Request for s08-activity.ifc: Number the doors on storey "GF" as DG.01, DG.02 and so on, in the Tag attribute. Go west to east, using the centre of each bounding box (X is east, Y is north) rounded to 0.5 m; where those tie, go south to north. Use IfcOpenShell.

First a look at what the model holds.

```python
import ifcopenshell
import ifcopenshell.util.element
import ifcopenshell.util.placement

model = ifcopenshell.open("s08-activity.ifc")
print(model.schema)
storey = next(s for s in model.by_type("IfcBuildingStorey") if s.Name == "GF")
doors = [e for e in ifcopenshell.util.element.get_decomposition(storey) if e.is_a("IfcDoor")]
for e in sorted(doors, key=lambda e: e.id()):
    origin = ifcopenshell.util.placement.get_local_placement(e.ObjectPlacement)[:3, 3]
    print(e.id(), e.Tag, e.Name, origin.round(2) + 0.0, sep=" | ")
```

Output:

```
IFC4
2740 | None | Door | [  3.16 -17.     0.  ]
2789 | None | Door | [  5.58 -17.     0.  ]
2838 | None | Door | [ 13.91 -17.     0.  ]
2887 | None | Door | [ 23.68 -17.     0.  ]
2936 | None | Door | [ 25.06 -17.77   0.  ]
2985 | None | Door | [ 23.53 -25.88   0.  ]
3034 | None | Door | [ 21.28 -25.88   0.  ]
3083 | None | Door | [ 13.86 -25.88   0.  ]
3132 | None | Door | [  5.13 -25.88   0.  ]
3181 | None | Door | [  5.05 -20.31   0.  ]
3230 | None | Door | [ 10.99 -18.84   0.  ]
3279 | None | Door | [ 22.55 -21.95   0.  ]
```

```python
import ifcopenshell
import ifcopenshell.geom
import ifcopenshell.util.element
import ifcopenshell.util.shape

model = ifcopenshell.open("s08-activity.ifc")
settings = ifcopenshell.geom.settings()
settings.set("use-world-coords", True)


def centre(element):
    shape = ifcopenshell.geom.create_shape(settings, element)
    return ifcopenshell.util.shape.get_bbox_centroid(shape.geometry)


storey = next(s for s in model.by_type("IfcBuildingStorey") if s.Name == "GF")
doors = [e for e in ifcopenshell.util.element.get_decomposition(storey) if e.is_a("IfcDoor")]

# Insertion points can sit at a corner or the storey origin, so sort by the geometry (in metres).
centres = {e: centre(e) for e in doors}
doors.sort(key=lambda e: (round(centres[e][0] / 0.5), centres[e][1]))

for i, e in enumerate(doors, start=1):
    number = f"DG.{i:02d}"
    e.Tag = number
    print(e.id(), number)

model.write("s08-activity_updated.ifc")
```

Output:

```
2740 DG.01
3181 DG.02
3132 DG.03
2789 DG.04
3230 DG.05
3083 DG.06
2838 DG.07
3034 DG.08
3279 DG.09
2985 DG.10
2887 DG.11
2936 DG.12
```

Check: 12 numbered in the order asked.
